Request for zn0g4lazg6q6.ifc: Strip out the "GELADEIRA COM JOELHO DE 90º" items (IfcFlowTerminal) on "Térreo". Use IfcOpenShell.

First a look at what the model holds.

```python
import ifcopenshell
import ifcopenshell.util.element

model = ifcopenshell.open("zn0g4lazg6q6.ifc")
print(model.schema)
storey = next(s for s in model.by_type("IfcBuildingStorey") if s.Name == "Térreo")
terminals = [e for e in ifcopenshell.util.element.get_decomposition(storey) if e.is_a("IfcFlowTerminal")]
seen = {}
for e in terminals:
    element_type = ifcopenshell.util.element.get_type(e)
    name = element_type.Name if element_type not in (None, e) else None
    seen[name] = seen.get(name, 0) + 1
for name, count in sorted(seen.items(), key=str):
    print(count, "x", name)
```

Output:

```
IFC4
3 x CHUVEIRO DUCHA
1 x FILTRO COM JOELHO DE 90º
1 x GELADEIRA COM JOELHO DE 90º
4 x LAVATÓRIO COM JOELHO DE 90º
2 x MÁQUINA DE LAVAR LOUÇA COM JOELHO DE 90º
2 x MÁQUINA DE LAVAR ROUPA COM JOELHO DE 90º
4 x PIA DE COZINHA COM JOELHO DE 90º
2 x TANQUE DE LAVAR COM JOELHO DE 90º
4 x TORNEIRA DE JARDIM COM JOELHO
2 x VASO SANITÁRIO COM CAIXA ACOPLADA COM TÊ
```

```python
import ifcopenshell
import ifcopenshell.api.root
import ifcopenshell.util.element

model = ifcopenshell.open("zn0g4lazg6q6.ifc")

storey = next(s for s in model.by_type("IfcBuildingStorey") if s.Name == "Térreo")
terminals = [e for e in ifcopenshell.util.element.get_decomposition(storey) if e.is_a("IfcFlowTerminal")]
targets = [e for e in terminals if (t := ifcopenshell.util.element.get_type(e)) not in (None, e) and t.Name == "GELADEIRA COM JOELHO DE 90º"]

for e in targets:
    ifcopenshell.api.root.remove_product(model, product=e)
print(len(targets), "removed")

model.write("zn0g4lazg6q6_rev.ifc")
```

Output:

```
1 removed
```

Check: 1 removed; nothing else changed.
